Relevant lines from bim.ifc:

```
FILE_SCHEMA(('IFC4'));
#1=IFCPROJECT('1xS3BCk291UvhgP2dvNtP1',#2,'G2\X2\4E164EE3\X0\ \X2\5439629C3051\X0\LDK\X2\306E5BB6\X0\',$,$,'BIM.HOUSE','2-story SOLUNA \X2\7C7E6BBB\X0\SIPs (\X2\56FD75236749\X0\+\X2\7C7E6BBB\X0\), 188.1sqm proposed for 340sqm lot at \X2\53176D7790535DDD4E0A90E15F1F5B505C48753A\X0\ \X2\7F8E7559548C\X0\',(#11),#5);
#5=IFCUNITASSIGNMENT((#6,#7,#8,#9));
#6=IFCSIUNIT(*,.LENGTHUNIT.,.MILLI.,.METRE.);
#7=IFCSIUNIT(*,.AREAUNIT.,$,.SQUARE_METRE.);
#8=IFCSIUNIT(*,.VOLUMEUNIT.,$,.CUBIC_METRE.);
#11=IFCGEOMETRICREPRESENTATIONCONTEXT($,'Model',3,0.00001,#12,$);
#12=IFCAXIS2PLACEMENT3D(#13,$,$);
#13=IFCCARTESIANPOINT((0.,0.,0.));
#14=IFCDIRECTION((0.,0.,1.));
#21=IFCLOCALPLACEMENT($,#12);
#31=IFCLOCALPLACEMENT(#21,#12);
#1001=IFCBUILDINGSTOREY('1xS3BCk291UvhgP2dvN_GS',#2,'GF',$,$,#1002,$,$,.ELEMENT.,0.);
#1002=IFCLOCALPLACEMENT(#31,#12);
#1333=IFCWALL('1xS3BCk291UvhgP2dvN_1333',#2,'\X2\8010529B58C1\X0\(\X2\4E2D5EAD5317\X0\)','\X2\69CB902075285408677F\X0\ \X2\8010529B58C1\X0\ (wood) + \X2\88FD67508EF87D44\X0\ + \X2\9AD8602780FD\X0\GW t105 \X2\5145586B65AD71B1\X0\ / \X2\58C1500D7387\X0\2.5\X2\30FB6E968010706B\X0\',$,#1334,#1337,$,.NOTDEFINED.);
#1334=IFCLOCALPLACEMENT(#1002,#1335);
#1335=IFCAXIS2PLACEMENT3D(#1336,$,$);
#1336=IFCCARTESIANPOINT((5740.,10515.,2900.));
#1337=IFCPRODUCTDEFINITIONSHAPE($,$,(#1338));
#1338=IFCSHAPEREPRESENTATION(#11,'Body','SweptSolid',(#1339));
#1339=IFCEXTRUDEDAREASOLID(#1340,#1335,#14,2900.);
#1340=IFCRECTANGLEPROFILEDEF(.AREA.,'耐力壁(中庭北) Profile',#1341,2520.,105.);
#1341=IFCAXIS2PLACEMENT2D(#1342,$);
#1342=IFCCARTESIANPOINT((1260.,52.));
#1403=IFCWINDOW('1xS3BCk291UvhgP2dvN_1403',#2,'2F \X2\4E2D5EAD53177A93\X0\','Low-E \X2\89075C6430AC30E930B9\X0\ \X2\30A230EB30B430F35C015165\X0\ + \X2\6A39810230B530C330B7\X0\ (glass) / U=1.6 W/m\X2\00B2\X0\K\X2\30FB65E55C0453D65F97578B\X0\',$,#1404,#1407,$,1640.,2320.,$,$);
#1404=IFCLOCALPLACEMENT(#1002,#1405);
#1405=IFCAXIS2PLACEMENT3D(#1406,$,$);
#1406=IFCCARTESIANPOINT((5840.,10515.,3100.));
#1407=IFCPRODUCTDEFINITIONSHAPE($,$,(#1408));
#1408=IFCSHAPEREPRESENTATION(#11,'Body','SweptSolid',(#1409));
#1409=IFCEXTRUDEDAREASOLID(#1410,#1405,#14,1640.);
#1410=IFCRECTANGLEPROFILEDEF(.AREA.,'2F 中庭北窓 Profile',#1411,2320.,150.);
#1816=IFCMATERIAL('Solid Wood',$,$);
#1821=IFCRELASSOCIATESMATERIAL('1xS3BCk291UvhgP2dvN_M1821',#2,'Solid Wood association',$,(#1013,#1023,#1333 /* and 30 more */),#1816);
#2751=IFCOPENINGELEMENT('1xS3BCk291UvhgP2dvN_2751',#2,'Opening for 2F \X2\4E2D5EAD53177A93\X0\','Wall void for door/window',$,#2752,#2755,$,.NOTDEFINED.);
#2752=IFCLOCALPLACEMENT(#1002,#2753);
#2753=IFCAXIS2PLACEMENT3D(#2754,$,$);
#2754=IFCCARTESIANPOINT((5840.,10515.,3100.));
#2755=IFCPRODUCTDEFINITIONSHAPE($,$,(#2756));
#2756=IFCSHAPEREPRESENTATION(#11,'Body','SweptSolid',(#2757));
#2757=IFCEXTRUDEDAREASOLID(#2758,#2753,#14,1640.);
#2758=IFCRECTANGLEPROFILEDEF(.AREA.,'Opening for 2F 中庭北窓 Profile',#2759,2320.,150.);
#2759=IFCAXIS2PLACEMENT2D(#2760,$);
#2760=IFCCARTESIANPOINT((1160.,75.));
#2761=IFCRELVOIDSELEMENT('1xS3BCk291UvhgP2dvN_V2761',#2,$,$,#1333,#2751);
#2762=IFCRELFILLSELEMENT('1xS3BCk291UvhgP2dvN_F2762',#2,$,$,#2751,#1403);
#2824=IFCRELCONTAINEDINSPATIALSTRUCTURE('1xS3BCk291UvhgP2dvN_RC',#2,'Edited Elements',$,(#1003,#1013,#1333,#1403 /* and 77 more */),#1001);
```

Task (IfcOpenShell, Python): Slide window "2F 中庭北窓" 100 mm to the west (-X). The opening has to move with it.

```python
import ifcopenshell
import ifcopenshell.api.geometry
import ifcopenshell.util.placement

model = ifcopenshell.open("bim.ifc")

window = model.by_guid("1xS3BCk291UvhgP2dvN_1403")
opening = window.FillsVoids[0].RelatingOpeningElement
wall = opening.VoidsElements[0].RelatingBuildingElement

wall_matrix = ifcopenshell.util.placement.get_local_placement(wall.ObjectPlacement)
shift = wall_matrix[:3, 0] * -100.0
before = ifcopenshell.util.placement.get_local_placement(window.ObjectPlacement)[:3, 3].copy()

# The window is not placed relative to its opening, so move both.
for product in (opening, window):
    matrix = ifcopenshell.util.placement.get_local_placement(product.ObjectPlacement)
    matrix[:3, 3] += shift
    ifcopenshell.api.geometry.edit_object_placement(model, product=product, matrix=matrix, is_si=False)

after = ifcopenshell.util.placement.get_local_placement(window.ObjectPlacement)[:3, 3]
print("window moved by", (after - before).round(3) + 0.0)

model.write("bim_edited.ifc")
```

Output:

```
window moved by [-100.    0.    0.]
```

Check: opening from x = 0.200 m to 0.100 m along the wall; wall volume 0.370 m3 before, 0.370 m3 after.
